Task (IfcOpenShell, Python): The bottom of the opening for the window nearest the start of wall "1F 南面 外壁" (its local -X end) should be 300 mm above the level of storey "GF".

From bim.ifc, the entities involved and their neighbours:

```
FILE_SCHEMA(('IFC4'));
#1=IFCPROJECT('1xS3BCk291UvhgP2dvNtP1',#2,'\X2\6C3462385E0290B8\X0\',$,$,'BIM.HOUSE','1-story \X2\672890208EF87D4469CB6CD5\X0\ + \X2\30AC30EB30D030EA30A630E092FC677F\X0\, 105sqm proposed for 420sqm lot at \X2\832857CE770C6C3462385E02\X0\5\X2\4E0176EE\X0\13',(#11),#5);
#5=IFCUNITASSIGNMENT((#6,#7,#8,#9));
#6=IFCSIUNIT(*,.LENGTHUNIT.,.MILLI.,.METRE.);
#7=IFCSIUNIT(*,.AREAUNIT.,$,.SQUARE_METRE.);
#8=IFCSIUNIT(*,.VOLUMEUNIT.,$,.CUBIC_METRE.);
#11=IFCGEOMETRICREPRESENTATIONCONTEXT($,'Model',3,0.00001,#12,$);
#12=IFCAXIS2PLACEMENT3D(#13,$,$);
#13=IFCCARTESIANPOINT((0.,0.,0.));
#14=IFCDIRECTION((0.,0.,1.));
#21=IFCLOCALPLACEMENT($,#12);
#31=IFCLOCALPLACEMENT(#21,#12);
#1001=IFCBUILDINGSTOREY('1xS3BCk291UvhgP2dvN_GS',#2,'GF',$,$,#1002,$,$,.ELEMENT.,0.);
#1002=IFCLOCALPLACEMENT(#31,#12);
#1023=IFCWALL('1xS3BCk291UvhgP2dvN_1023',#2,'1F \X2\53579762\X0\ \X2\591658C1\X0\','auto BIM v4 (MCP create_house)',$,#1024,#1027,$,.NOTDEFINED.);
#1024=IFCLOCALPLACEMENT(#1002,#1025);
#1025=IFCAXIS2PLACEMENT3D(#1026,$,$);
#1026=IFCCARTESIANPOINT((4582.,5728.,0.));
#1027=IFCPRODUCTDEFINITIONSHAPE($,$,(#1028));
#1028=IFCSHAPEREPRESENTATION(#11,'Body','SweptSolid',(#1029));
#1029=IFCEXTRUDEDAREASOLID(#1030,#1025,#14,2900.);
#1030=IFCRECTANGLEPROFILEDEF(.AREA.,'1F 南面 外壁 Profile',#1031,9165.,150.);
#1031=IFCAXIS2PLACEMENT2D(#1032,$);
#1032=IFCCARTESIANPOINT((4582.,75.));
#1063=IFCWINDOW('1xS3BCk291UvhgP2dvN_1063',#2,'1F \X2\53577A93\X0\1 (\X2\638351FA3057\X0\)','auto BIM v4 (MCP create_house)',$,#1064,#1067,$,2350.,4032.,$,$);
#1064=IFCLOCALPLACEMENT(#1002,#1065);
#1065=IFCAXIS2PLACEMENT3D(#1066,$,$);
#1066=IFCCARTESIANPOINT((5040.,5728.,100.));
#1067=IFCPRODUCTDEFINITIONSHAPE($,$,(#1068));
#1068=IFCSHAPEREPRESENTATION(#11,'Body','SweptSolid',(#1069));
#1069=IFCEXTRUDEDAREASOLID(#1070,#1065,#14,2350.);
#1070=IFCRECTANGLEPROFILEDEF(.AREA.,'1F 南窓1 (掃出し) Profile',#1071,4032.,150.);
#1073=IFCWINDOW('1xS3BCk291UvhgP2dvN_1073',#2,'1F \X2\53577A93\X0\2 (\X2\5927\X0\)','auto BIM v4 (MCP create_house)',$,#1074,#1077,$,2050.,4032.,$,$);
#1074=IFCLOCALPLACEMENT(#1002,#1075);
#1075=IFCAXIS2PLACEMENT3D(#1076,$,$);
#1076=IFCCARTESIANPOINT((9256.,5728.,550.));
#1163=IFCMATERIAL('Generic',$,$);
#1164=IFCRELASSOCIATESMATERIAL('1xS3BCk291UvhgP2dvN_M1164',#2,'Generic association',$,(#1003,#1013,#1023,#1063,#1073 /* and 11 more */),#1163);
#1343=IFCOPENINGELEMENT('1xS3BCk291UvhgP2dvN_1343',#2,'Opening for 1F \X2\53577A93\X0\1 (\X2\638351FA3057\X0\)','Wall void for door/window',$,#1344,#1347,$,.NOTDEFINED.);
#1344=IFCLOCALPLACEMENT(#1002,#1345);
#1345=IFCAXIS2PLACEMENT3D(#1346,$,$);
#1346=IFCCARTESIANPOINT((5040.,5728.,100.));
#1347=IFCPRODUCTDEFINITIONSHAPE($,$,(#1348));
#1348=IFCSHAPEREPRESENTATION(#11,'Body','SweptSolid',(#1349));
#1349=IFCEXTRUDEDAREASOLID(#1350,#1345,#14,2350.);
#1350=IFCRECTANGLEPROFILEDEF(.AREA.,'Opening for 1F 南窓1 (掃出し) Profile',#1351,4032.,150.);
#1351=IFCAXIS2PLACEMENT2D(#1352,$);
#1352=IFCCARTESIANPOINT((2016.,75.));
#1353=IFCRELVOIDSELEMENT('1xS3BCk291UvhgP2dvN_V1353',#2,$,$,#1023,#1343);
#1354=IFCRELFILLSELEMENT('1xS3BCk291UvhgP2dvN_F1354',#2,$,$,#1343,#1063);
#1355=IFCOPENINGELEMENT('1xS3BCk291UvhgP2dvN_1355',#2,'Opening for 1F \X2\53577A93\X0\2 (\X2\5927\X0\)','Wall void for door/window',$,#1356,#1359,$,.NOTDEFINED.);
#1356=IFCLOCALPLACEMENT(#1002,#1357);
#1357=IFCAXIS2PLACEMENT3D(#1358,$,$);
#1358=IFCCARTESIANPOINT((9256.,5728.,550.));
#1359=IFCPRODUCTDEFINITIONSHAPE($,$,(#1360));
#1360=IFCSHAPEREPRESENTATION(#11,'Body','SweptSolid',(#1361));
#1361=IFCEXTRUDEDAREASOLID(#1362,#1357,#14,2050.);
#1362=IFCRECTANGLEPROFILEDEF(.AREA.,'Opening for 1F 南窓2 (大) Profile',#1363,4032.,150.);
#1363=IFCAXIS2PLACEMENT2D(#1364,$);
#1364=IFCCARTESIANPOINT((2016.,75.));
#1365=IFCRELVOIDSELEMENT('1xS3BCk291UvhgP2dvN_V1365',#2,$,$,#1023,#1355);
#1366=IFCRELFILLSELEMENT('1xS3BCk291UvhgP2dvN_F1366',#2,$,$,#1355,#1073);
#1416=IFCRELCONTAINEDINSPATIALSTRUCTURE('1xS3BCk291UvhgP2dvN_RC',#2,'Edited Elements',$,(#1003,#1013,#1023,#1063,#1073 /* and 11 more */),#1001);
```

```python
import numpy as np
import ifcopenshell
import ifcopenshell.api.geometry
import ifcopenshell.geom
import ifcopenshell.util.element
import ifcopenshell.util.placement
import ifcopenshell.util.shape
import ifcopenshell.util.unit

model = ifcopenshell.open("bim.ifc")
unit_scale = ifcopenshell.util.unit.calculate_unit_scale(model)

window = model.by_id(1063)
opening = window.FillsVoids[0].RelatingOpeningElement
storey = ifcopenshell.util.element.get_container(window, ifc_class="IfcBuildingStorey")
level = ifcopenshell.util.placement.get_local_placement(storey.ObjectPlacement)[2, 3]

# The opening's origin need not be at the sill, so measure its lowest point.
shape = ifcopenshell.geom.create_shape(ifcopenshell.geom.settings(), opening)
bottom = ifcopenshell.util.shape.get_shape_bottom_elevation(shape, shape.geometry) / unit_scale
dz = level + 0.3 / unit_scale - bottom

shift = np.array([0.0, 0.0, dz])
# The window is not placed relative to its opening, so move both.
for product in (opening, window):
    matrix = ifcopenshell.util.placement.get_local_placement(product.ObjectPlacement)
    matrix[:3, 3] += shift
    ifcopenshell.api.geometry.edit_object_placement(model, product=product, matrix=matrix, is_si=False)

print(f"moved by {dz * unit_scale:+.3f} m")

model.write("bim-out.ifc")
```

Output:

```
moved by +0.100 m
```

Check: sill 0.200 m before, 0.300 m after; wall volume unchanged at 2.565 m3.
